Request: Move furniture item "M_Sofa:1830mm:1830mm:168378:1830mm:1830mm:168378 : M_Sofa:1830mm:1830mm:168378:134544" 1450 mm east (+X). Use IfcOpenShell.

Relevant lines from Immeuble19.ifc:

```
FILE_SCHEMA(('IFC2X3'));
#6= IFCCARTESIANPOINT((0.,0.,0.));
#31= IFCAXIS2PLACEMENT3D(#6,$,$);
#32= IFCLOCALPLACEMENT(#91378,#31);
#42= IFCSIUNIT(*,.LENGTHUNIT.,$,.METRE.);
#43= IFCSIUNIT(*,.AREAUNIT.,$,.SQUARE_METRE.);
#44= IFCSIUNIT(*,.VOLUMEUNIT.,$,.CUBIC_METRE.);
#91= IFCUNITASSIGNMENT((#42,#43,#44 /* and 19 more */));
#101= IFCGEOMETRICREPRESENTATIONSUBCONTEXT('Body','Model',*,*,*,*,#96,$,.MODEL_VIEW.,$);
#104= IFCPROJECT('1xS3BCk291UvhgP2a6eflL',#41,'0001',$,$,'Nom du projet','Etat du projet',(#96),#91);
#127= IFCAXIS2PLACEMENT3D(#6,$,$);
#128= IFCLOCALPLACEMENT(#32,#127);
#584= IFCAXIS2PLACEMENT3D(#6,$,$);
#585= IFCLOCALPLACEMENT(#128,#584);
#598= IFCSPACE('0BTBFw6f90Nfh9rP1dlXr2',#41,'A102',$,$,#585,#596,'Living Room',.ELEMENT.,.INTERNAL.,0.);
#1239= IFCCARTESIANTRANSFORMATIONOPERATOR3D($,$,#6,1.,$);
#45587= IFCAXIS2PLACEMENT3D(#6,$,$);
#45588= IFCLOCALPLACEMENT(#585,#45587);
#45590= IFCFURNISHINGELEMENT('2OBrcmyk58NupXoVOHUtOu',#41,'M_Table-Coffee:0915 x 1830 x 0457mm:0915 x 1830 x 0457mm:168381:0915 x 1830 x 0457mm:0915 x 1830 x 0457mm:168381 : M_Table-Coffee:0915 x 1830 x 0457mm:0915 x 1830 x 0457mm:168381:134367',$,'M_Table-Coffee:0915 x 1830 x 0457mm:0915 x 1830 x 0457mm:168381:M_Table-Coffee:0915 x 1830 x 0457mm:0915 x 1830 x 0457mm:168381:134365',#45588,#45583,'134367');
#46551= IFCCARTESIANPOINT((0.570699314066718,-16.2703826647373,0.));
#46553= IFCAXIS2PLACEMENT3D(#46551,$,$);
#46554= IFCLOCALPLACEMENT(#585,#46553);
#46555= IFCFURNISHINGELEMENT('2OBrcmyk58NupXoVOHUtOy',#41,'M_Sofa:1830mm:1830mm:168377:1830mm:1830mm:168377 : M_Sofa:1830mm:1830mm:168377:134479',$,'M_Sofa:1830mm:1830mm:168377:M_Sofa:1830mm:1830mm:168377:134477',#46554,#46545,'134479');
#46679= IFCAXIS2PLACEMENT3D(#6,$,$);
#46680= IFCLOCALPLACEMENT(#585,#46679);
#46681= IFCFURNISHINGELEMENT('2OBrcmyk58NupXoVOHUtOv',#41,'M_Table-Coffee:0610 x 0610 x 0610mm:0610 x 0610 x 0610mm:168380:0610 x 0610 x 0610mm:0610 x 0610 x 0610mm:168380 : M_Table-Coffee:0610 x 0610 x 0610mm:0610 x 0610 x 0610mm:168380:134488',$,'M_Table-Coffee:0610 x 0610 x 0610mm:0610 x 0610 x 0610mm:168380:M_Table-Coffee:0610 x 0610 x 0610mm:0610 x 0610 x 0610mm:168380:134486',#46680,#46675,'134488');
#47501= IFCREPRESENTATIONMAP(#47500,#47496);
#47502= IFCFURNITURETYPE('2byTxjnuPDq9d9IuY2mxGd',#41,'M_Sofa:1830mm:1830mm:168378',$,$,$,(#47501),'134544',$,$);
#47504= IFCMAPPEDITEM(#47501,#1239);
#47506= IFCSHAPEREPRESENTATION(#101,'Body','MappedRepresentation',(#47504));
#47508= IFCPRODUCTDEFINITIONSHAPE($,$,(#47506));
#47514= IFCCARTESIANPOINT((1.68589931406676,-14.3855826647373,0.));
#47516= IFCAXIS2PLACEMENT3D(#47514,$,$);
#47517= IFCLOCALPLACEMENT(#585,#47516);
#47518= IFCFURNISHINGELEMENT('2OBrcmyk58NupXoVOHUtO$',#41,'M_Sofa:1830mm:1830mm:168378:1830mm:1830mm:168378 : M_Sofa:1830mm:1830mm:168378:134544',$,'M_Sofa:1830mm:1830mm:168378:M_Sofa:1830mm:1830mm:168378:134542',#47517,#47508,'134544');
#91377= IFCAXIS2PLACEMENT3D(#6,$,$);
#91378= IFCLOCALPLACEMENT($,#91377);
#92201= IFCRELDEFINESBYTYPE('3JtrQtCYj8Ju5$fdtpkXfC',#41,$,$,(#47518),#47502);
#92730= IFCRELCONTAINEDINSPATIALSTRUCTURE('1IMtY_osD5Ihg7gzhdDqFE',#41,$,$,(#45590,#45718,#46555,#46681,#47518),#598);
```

```python
import ifcopenshell
import ifcopenshell.api.geometry
import ifcopenshell.util.placement
import ifcopenshell.util.unit

model = ifcopenshell.open("Immeuble19.ifc")
unit_scale = ifcopenshell.util.unit.calculate_unit_scale(model)

item = model.by_guid("2OBrcmyk58NupXoVOHUtO$")
matrix = ifcopenshell.util.placement.get_local_placement(item.ObjectPlacement)
matrix[0, 3] += 1.45 / unit_scale
ifcopenshell.api.geometry.edit_object_placement(model, product=item, matrix=matrix, is_si=False)

print(ifcopenshell.util.placement.get_local_placement(item.ObjectPlacement).round(3) + 0.0)

model.write("Immeuble19_edited.ifc")
```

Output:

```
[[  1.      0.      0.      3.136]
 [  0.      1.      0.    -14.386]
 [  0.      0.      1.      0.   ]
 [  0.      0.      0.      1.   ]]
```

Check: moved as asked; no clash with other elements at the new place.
